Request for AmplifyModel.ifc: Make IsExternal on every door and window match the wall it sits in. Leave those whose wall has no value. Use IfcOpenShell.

First a look at what the model holds.

```python
import ifcopenshell
import ifcopenshell.util.element

model = ifcopenshell.open("AmplifyModel.ifc")
print(model.schema)
seen = {}
for e in model.by_type("IfcDoor") + model.by_type("IfcWindow"):
    if not e.FillsVoids:
        continue
    host = e.FillsVoids[0].RelatingOpeningElement.VoidsElements[0].RelatingBuildingElement
    own = ifcopenshell.util.element.get_pset(e, f"Pset_{e.is_a()[3:].removesuffix('StandardCase')}Common", "IsExternal")
    wall = ifcopenshell.util.element.get_pset(host, "Pset_WallCommon", "IsExternal")
    seen[e.is_a(), own, wall] = seen.get((e.is_a(), own, wall), 0) + 1
for (cls, own, wall), count in sorted(seen.items(), key=str):
    print(count, cls, "IsExternal:", own, "| host wall:", wall)
```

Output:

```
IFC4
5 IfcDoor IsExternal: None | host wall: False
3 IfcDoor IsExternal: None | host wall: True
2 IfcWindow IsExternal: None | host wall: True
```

```python
import ifcopenshell
import ifcopenshell.api.pset
import ifcopenshell.util.element

model = ifcopenshell.open("AmplifyModel.ifc")

count = 0
for ifc_class, pset_name in (("IfcDoor", "Pset_DoorCommon"), ("IfcWindow", "Pset_WindowCommon")):
    for e in model.by_type(ifc_class):
        if not e.FillsVoids:
            continue
        host = e.FillsVoids[0].RelatingOpeningElement.VoidsElements[0].RelatingBuildingElement
        external = ifcopenshell.util.element.get_pset(host, "Pset_WallCommon", "IsExternal")
        if external is None or ifcopenshell.util.element.get_pset(e, pset_name, "IsExternal") == external:
            continue
        pset = ifcopenshell.api.pset.add_pset(model, product=e, name=pset_name)
        ifcopenshell.api.pset.edit_pset(model, pset=pset, properties={"IsExternal": external})
        count += 1

print(count, "updated")

model.write("AmplifyModel_rev.ifc")
```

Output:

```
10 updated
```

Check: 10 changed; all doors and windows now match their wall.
